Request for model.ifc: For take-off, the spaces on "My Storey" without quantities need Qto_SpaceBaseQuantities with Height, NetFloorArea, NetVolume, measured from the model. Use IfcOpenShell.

First a look at what the model holds.

```python
import ifcopenshell
import ifcopenshell.util.element
import ifcopenshell.util.unit

model = ifcopenshell.open("model.ifc")
print(model.schema)
for unit_type in ("LENGTHUNIT", "AREAUNIT", "VOLUMEUNIT"):
    print(unit_type, ifcopenshell.util.unit.calculate_unit_scale(model, unit_type))
storey = next(s for s in model.by_type("IfcBuildingStorey") if s.Name == "My Storey")
spaces = [e for e in ifcopenshell.util.element.get_decomposition(storey) if e.is_a("IfcSpace")]
for e in sorted(spaces, key=lambda e: e.id()):
    print(e.id(), e.is_a(), e.Name, list(ifcopenshell.util.element.get_psets(e, qtos_only=True)), sep=" | ")
```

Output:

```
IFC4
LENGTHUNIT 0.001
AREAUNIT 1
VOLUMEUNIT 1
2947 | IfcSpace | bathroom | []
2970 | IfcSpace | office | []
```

```python
import ifcopenshell
import ifcopenshell.api.pset
import ifcopenshell.geom
import ifcopenshell.util.element
import ifcopenshell.util.shape
import ifcopenshell.util.unit

model = ifcopenshell.open("model.ifc")
unit_scale = ifcopenshell.util.unit.calculate_unit_scale(model)
area_scale = ifcopenshell.util.unit.calculate_unit_scale(model, "AREAUNIT")
volume_scale = ifcopenshell.util.unit.calculate_unit_scale(model, "VOLUMEUNIT")
settings = ifcopenshell.geom.settings()

storey = next(s for s in model.by_type("IfcBuildingStorey") if s.Name == "My Storey")
spaces = [e for e in ifcopenshell.util.element.get_decomposition(storey) if e.is_a("IfcSpace")]

for e in sorted(spaces, key=lambda e: e.id()):
    if ifcopenshell.util.element.get_psets(e, qtos_only=True, should_inherit=False):
        continue
    # Geometry comes back in metres, in the element's own axes.
    shape = ifcopenshell.geom.create_shape(settings, e)
    values = {
        "Height": ifcopenshell.util.shape.get_z(shape.geometry) / unit_scale,
        "NetFloorArea": ifcopenshell.util.shape.get_footprint_area(shape.geometry) / area_scale,
        "NetVolume": ifcopenshell.util.shape.get_volume(shape.geometry) / volume_scale,
    }
    qto = ifcopenshell.api.pset.add_qto(model, product=e, name="Qto_SpaceBaseQuantities")
    ifcopenshell.api.pset.edit_qto(model, qto=qto, properties=values)
    print(e.id(), {k: round(v, 3) for k, v in values.items()})

model.write("model-out.ifc")
```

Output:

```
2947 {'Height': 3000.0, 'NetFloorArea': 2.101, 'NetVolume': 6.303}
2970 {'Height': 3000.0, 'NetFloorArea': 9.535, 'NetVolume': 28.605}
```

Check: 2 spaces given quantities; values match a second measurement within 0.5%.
